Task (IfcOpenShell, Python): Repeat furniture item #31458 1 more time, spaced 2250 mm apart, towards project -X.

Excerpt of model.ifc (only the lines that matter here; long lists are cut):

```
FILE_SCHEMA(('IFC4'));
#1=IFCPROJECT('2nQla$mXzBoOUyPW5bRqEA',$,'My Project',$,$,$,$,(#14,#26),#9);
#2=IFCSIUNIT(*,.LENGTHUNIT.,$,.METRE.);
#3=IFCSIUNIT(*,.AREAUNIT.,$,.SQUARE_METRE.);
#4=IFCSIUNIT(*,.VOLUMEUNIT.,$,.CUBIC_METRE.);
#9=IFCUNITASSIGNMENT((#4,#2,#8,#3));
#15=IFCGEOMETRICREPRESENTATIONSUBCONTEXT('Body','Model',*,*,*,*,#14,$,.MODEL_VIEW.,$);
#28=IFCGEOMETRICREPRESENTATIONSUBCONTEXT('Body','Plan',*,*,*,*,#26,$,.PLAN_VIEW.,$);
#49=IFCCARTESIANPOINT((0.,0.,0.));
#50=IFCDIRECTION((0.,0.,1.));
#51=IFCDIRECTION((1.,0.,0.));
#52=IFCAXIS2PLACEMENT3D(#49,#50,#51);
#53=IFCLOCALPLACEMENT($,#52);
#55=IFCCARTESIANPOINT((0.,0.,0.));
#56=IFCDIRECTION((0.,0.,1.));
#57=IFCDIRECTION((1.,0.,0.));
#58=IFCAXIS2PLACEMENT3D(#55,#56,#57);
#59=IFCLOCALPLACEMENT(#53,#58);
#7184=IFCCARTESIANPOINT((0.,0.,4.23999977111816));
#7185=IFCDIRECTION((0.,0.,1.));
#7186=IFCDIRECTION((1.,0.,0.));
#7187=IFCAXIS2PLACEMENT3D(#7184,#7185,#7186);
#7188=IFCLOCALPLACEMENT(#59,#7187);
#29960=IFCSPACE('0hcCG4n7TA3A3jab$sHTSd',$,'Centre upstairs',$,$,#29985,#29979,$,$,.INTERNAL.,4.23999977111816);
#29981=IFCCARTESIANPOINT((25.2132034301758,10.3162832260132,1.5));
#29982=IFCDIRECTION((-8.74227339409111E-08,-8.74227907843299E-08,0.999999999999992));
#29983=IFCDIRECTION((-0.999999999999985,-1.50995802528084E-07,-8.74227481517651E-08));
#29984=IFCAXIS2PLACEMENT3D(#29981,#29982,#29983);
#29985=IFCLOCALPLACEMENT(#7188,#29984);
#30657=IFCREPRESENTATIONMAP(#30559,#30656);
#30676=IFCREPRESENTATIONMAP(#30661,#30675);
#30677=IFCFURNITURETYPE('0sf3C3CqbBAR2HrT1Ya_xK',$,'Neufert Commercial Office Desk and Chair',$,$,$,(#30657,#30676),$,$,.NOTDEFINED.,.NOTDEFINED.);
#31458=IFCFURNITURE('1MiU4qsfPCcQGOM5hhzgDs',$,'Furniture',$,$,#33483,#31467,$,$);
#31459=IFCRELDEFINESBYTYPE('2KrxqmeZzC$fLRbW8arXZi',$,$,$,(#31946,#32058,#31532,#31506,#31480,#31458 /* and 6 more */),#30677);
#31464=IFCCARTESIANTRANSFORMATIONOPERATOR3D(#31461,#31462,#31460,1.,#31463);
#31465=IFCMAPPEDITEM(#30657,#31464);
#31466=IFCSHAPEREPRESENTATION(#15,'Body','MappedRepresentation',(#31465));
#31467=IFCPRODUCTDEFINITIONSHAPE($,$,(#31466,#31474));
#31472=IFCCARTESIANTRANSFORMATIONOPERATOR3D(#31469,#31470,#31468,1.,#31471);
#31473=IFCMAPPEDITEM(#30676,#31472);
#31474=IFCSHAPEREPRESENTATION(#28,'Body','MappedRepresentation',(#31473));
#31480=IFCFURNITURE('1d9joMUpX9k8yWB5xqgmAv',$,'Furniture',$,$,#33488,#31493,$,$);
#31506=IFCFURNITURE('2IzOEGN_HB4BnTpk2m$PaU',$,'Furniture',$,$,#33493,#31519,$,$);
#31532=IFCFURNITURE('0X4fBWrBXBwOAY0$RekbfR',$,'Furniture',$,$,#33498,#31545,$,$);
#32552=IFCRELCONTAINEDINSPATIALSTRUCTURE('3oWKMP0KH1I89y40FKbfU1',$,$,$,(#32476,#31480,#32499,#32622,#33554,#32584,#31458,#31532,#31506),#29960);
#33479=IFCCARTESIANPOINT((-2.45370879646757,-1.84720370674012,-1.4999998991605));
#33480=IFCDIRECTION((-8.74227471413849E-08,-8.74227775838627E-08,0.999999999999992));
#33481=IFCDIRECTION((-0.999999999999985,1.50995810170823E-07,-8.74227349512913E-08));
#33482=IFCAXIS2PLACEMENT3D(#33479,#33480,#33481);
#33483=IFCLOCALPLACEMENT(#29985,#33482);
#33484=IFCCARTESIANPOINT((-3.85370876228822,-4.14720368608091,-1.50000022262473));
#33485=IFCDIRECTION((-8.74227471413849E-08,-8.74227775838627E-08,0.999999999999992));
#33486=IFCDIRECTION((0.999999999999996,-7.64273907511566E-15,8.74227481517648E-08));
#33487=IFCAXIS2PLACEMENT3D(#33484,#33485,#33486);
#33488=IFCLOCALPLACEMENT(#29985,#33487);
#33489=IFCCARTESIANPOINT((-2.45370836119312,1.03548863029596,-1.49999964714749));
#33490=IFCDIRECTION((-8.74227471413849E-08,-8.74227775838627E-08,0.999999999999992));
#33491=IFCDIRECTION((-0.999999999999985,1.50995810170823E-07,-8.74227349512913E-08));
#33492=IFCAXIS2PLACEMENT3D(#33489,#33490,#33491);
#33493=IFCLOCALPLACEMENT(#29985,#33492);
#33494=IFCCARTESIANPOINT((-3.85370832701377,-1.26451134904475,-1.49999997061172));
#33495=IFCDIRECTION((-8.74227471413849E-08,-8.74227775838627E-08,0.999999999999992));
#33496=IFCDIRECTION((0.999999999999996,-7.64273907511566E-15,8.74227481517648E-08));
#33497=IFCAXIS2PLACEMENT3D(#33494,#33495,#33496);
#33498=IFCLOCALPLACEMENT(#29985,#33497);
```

```python
import numpy as np
import ifcopenshell
import ifcopenshell.api.geometry
import ifcopenshell.api.root
import ifcopenshell.util.element
import ifcopenshell.util.placement
import ifcopenshell.util.unit

model = ifcopenshell.open("model.ifc")
unit_scale = ifcopenshell.util.unit.calculate_unit_scale(model)

source = model.by_id(31458)
base = ifcopenshell.util.placement.get_local_placement(source.ObjectPlacement)
step = np.array([-1.0, 0.0, 0.0]) * 2.25 / unit_scale

for i in range(1, 2):
    copy = ifcopenshell.api.root.copy_class(model, product=source)
    copy.Representation = ifcopenshell.util.element.copy_deep(
        model, source.Representation, exclude=["IfcGeometricRepresentationContext", "IfcRepresentationMap"]
    )
    matrix = base.copy()
    matrix[:3, 3] += i * step
    print("added at", matrix[:3, 3].round(3) + 0.0)
    ifcopenshell.api.geometry.edit_object_placement(model, product=copy, matrix=matrix, is_si=False)

model.write("model_edited.ifc")
```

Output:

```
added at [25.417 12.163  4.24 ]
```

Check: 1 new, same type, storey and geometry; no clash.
